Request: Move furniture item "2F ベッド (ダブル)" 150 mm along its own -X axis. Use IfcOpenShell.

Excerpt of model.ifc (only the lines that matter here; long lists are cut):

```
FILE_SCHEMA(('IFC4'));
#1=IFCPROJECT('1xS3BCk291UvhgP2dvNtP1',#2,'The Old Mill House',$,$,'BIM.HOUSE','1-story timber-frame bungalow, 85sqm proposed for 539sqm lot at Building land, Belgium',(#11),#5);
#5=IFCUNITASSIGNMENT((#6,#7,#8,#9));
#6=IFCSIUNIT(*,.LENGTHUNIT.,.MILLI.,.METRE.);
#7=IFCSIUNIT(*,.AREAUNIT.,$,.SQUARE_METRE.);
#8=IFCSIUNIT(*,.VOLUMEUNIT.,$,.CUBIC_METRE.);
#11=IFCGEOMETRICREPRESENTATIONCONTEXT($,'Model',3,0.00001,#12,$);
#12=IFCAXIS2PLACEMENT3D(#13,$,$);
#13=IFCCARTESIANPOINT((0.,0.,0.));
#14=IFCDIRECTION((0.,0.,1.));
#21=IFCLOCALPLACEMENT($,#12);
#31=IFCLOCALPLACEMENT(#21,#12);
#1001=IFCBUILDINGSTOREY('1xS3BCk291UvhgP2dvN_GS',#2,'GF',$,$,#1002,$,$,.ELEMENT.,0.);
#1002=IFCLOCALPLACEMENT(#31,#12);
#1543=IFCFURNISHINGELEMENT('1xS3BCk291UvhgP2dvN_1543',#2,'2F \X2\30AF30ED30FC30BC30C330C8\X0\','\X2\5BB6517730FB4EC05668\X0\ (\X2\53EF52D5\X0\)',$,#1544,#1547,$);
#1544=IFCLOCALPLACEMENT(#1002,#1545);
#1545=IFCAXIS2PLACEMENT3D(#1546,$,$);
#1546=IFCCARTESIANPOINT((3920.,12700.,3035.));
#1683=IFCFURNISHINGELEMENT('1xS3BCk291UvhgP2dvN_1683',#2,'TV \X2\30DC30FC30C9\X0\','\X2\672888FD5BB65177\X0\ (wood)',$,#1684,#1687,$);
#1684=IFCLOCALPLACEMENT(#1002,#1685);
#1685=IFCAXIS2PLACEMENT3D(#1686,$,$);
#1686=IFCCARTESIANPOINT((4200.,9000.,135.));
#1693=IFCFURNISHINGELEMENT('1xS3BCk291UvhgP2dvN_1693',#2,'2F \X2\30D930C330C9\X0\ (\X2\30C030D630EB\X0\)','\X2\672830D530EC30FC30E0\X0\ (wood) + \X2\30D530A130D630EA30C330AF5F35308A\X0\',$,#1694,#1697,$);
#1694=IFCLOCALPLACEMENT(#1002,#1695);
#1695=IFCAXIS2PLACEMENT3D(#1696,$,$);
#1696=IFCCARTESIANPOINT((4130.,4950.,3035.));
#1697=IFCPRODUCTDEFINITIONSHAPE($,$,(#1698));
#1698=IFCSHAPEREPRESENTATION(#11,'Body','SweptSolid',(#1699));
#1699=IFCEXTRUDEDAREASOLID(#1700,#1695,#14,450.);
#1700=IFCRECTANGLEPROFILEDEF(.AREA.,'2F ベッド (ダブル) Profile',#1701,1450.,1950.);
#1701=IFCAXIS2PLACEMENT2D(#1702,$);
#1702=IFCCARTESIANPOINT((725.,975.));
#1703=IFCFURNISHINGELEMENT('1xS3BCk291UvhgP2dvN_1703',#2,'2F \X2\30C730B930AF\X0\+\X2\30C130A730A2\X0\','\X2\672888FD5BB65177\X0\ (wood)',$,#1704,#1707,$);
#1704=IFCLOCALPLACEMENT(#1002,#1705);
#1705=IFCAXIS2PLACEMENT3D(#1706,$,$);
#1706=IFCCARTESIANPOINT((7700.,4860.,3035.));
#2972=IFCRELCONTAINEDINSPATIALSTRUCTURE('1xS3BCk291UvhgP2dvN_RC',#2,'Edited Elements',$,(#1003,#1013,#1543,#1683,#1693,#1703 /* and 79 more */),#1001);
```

```python
import ifcopenshell
import ifcopenshell.api.geometry
import ifcopenshell.util.placement

model = ifcopenshell.open("model.ifc")

item = model.by_guid("1xS3BCk291UvhgP2dvN_1693")
matrix = ifcopenshell.util.placement.get_local_placement(item.ObjectPlacement)
matrix[:3, 3] -= matrix[:3, 0] * 150.0
ifcopenshell.api.geometry.edit_object_placement(model, product=item, matrix=matrix, is_si=False)

print(ifcopenshell.util.placement.get_local_placement(item.ObjectPlacement).round(3) + 0.0)

model.write("model-out.ifc")
```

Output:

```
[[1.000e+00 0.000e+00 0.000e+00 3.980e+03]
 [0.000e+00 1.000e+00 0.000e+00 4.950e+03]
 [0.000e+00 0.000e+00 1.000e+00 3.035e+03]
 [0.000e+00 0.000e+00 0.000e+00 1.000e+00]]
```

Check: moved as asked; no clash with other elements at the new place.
